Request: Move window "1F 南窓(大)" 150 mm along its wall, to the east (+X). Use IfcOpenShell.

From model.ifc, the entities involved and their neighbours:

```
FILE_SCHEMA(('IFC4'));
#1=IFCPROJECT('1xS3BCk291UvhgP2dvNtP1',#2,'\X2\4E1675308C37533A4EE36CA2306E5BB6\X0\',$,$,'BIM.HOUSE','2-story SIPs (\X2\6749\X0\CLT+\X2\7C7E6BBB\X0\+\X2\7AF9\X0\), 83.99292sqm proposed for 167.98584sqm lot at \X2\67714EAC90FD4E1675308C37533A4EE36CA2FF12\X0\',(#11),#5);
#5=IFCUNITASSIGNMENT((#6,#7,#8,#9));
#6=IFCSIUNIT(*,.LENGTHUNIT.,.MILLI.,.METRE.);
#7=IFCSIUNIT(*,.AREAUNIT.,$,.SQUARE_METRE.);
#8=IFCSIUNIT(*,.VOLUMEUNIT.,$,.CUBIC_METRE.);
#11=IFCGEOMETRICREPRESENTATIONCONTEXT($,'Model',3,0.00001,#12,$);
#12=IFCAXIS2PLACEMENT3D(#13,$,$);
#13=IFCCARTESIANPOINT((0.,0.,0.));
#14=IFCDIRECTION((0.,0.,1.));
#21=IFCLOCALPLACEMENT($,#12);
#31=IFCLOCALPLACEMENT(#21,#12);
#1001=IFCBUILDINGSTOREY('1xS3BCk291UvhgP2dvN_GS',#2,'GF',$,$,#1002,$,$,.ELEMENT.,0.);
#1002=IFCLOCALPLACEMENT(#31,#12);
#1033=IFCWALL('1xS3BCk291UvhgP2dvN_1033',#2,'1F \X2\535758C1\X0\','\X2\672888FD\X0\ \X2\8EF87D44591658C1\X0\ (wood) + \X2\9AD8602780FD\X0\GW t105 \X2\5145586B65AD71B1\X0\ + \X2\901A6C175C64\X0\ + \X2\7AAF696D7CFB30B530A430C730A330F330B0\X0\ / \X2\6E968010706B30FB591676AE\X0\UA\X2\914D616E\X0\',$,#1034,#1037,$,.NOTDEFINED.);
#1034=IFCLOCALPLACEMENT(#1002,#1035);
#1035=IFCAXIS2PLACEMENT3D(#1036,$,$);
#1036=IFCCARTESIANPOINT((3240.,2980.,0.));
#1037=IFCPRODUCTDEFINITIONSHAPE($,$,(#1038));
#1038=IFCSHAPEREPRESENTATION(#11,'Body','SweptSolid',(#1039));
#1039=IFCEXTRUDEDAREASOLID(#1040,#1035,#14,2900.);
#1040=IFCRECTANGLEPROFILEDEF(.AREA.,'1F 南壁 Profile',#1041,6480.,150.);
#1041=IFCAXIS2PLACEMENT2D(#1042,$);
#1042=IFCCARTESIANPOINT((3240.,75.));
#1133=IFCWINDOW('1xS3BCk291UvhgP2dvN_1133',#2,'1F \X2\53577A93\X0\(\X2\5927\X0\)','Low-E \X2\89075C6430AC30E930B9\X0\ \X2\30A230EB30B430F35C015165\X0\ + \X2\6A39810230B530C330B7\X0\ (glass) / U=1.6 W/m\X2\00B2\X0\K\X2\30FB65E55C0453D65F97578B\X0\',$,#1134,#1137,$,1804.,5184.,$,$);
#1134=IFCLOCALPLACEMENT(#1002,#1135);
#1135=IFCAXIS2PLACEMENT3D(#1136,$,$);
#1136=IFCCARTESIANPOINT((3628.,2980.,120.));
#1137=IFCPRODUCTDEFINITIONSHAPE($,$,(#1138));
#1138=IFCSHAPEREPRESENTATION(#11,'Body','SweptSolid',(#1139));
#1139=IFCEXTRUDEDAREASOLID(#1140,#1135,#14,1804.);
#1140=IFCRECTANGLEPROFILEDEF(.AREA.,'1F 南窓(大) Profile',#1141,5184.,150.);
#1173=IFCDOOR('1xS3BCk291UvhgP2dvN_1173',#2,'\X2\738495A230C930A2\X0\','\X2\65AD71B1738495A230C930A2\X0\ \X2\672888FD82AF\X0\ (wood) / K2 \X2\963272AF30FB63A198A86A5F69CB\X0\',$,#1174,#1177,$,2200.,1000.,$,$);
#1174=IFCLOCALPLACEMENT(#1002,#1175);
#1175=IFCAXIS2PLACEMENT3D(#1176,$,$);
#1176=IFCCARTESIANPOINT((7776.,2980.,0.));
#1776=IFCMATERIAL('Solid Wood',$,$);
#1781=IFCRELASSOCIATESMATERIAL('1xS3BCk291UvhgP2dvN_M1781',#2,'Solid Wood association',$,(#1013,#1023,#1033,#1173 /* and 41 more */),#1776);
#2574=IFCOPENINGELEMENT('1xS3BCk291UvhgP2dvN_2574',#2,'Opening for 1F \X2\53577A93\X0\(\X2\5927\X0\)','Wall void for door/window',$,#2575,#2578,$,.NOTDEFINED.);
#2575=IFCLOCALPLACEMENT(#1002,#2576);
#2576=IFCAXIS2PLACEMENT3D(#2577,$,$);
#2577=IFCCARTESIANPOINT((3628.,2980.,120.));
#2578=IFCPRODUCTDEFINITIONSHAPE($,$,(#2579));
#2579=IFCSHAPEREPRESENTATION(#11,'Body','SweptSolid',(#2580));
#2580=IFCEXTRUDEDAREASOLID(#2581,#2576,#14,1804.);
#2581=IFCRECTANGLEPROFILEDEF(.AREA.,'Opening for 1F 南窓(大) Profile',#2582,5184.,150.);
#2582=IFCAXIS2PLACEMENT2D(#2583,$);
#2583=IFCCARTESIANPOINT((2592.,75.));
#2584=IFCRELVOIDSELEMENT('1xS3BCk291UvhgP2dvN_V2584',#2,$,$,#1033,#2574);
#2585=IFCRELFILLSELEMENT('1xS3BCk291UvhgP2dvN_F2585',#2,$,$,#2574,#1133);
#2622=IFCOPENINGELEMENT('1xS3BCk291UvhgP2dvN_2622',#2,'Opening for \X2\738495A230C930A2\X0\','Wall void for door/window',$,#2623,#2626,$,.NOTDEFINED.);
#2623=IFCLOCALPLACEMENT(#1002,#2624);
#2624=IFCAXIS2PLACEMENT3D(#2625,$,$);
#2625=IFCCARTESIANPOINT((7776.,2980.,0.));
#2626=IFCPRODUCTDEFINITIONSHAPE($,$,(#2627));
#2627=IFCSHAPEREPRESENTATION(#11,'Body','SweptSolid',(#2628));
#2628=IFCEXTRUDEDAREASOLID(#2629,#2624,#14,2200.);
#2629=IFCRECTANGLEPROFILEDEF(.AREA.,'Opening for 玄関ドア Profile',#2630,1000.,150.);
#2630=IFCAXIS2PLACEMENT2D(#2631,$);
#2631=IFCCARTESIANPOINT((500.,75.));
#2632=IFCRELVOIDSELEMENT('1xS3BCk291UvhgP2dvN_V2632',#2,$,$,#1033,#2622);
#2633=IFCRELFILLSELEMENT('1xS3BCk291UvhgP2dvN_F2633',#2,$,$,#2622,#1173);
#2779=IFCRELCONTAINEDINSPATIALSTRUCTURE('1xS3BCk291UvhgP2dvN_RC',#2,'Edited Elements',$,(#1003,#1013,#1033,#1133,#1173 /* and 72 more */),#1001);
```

```python
import ifcopenshell
import ifcopenshell.api.geometry
import ifcopenshell.util.placement
import ifcopenshell.util.unit

model = ifcopenshell.open("model.ifc")
unit_scale = ifcopenshell.util.unit.calculate_unit_scale(model)

window = model.by_guid("1xS3BCk291UvhgP2dvN_1133")
opening = window.FillsVoids[0].RelatingOpeningElement
wall = opening.VoidsElements[0].RelatingBuildingElement

wall_matrix = ifcopenshell.util.placement.get_local_placement(wall.ObjectPlacement)
shift = wall_matrix[:3, 0] * 0.15 / unit_scale
before = ifcopenshell.util.placement.get_local_placement(window.ObjectPlacement)[:3, 3].copy()

# The window is not placed relative to its opening, so move both.
for product in (opening, window):
    matrix = ifcopenshell.util.placement.get_local_placement(product.ObjectPlacement)
    matrix[:3, 3] += shift
    ifcopenshell.api.geometry.edit_object_placement(model, product=product, matrix=matrix, is_si=False)

after = ifcopenshell.util.placement.get_local_placement(window.ObjectPlacement)[:3, 3]
print("window moved by", (after - before).round(3) + 0.0)

model.write("model_rev.ifc")
```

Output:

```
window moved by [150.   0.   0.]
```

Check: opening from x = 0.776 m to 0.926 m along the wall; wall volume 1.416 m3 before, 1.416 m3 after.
